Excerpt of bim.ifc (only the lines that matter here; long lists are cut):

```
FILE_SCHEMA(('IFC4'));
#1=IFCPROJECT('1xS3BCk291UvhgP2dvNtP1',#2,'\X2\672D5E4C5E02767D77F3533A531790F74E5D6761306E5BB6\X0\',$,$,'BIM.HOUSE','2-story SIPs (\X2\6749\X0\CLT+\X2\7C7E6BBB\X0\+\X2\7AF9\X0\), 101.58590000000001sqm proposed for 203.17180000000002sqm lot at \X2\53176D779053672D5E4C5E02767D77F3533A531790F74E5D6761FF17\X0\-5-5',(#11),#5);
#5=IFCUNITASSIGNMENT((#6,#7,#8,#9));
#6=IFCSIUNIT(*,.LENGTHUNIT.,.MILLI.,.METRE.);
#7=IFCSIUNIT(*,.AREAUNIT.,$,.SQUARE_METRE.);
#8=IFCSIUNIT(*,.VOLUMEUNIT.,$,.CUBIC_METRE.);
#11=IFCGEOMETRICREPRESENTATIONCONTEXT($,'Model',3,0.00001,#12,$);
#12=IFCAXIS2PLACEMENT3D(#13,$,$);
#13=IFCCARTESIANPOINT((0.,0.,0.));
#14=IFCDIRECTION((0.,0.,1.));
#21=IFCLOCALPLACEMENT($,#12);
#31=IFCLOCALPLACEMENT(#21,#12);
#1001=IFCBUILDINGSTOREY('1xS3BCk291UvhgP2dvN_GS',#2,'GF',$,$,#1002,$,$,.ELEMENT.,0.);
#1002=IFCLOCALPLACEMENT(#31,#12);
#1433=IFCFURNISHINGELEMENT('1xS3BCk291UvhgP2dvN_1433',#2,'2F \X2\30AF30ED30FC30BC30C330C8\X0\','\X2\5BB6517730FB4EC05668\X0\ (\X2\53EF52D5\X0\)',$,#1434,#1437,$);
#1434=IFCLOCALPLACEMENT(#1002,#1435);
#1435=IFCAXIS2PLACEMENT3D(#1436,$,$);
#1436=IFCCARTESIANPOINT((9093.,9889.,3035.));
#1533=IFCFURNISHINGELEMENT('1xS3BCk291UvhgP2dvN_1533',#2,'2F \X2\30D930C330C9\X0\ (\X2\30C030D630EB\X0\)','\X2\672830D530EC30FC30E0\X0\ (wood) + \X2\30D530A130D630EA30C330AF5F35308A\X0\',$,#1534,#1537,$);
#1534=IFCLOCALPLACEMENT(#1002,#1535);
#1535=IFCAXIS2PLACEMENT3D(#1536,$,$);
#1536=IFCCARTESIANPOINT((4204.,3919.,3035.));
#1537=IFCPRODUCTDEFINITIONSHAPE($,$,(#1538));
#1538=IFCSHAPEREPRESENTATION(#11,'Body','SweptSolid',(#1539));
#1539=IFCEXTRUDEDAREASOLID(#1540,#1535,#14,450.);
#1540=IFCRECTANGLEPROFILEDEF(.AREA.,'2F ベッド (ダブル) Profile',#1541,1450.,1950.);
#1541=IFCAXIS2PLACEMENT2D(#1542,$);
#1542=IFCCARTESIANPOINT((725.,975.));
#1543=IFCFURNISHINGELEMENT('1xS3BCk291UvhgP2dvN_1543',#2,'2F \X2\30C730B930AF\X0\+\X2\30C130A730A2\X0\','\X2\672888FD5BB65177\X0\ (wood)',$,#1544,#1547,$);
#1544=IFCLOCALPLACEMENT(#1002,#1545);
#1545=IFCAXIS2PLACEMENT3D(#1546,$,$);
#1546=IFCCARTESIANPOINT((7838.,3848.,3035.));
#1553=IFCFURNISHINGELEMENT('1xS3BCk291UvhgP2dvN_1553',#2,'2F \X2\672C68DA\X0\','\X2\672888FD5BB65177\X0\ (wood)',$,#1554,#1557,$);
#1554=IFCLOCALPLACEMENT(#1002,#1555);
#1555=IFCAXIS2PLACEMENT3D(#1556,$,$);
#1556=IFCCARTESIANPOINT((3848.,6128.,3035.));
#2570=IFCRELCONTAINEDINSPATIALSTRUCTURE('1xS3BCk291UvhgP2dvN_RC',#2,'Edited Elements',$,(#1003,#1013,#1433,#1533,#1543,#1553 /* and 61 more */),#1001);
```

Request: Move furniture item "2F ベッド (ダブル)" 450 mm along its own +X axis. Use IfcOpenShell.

```python
import ifcopenshell
import ifcopenshell.api.geometry
import ifcopenshell.util.placement

model = ifcopenshell.open("bim.ifc")

item = model.by_guid("1xS3BCk291UvhgP2dvN_1533")
matrix = ifcopenshell.util.placement.get_local_placement(item.ObjectPlacement)
matrix[:3, 3] += matrix[:3, 0] * 450.0
ifcopenshell.api.geometry.edit_object_placement(model, product=item, matrix=matrix, is_si=False)

print(ifcopenshell.util.placement.get_local_placement(item.ObjectPlacement).round(3) + 0.0)

model.write("bim_edited.ifc")
```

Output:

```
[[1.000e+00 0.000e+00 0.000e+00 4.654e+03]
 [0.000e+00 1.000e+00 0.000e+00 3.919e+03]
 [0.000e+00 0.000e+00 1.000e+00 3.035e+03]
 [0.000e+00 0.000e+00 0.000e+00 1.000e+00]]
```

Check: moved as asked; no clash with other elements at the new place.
